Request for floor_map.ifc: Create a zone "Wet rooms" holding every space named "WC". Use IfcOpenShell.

First a look at what the model holds.

```python
import ifcopenshell

model = ifcopenshell.open("floor_map.ifc")
print(model.schema)
seen = {}
for space in model.by_type("IfcSpace"):
    seen[space.LongName] = seen.get(space.LongName, 0) + 1
for name, count in sorted(seen.items(), key=str):
    print(count, "x", name)
print("zones:", [z.Name for z in model.by_type("IfcZone")][:20])
```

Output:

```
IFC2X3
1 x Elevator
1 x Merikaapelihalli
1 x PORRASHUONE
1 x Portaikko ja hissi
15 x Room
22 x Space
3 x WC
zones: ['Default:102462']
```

```python
import ifcopenshell
import ifcopenshell.api.group
import ifcopenshell.api.root

model = ifcopenshell.open("floor_map.ifc")

names = {"WC"}
spaces = [s for s in model.by_type("IfcSpace") if s.LongName in names]

zone = ifcopenshell.api.root.create_entity(model, ifc_class="IfcZone", name="Wet rooms")
ifcopenshell.api.group.assign_group(model, products=spaces, group=zone)
print(len(spaces), "spaces in", zone.Name)

model.write("floor_map_edited.ifc")
```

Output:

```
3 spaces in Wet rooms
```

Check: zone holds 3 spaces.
